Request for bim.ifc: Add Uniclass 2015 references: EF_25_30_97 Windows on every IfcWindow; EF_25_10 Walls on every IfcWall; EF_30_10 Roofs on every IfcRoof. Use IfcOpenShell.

First a look at what the model holds.

```python
import ifcopenshell

model = ifcopenshell.open("bim.ifc")
print(model.schema)
print("classifications:", [c.Name for c in model.by_type("IfcClassification")])
for ifc_class in ("IfcDoor", "IfcRoof", "IfcStair", "IfcWall", "IfcWindow"):
    print(ifc_class, len(model.by_type(ifc_class)))
```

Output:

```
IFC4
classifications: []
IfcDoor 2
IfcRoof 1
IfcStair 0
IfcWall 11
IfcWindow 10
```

```python
import ifcopenshell
import ifcopenshell.api.classification

model = ifcopenshell.open("bim.ifc")

system = ifcopenshell.api.classification.add_classification(model, classification="Uniclass 2015")

codes = {
    "IfcWindow": ("EF_25_30_97", "Windows"),
    "IfcWall": ("EF_25_10", "Walls"),
    "IfcRoof": ("EF_30_10", "Roofs"),
}
for ifc_class, (code, name) in codes.items():
    products = model.by_type(ifc_class)
    ifcopenshell.api.classification.add_reference(
        model, products=products, classification=system, identification=code, name=name
    )
    print(code, len(products))

model.write("bim_edited.ifc")
```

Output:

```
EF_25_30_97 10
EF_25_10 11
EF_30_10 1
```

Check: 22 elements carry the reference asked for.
